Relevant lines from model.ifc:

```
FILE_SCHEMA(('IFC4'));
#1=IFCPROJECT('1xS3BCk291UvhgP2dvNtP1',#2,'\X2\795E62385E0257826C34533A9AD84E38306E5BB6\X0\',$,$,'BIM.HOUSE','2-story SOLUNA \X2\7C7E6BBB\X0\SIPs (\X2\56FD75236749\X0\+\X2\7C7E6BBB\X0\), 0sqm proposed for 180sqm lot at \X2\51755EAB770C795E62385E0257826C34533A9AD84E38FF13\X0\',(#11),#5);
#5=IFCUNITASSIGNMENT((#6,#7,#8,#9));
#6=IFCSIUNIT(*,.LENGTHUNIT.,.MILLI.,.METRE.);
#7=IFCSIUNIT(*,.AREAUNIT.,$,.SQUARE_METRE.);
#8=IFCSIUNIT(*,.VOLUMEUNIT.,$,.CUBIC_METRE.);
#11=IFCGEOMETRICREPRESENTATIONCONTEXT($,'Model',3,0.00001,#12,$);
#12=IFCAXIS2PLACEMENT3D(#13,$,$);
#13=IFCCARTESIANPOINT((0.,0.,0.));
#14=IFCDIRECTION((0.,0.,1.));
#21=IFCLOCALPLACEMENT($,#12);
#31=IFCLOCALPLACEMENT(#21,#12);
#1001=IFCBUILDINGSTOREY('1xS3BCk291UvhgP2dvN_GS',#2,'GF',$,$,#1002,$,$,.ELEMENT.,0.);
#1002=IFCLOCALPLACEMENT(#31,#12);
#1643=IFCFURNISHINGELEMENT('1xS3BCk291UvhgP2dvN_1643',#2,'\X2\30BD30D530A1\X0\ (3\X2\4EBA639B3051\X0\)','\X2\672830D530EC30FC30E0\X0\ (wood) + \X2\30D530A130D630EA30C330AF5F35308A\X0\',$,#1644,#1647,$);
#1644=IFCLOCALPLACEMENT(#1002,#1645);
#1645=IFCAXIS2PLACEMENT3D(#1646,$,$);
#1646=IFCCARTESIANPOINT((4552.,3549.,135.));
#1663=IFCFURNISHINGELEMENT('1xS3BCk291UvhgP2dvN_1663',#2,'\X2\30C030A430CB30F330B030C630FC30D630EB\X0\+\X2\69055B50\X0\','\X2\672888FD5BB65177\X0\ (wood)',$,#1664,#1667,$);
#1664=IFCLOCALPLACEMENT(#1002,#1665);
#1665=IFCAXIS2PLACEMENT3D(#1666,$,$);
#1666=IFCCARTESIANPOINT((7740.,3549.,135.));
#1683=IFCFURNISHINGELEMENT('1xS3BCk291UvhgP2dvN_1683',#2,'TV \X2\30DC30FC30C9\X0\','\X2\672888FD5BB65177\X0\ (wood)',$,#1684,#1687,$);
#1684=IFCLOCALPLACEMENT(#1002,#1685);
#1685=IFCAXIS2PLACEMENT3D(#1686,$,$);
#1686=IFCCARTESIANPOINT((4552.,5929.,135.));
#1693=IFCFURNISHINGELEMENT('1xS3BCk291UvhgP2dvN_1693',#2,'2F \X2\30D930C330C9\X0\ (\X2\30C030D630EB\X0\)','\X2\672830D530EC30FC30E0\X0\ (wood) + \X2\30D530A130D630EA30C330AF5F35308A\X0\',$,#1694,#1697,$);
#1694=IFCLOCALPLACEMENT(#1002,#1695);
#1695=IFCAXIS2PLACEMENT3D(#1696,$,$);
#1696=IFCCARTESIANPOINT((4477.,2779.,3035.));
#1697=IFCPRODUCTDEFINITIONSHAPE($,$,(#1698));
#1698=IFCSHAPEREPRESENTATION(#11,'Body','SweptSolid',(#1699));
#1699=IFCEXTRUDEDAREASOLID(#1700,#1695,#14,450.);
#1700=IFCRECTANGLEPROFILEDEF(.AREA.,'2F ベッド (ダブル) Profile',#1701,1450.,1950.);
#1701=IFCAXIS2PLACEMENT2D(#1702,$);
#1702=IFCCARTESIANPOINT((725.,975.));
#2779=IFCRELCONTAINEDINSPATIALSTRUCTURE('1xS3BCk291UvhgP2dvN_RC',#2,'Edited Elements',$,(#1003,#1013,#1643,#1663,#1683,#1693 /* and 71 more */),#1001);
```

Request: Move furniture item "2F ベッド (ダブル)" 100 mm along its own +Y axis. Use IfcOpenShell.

```python
import ifcopenshell
import ifcopenshell.api.geometry
import ifcopenshell.util.placement
import ifcopenshell.util.unit

model = ifcopenshell.open("model.ifc")
unit_scale = ifcopenshell.util.unit.calculate_unit_scale(model)

item = model.by_guid("1xS3BCk291UvhgP2dvN_1693")
matrix = ifcopenshell.util.placement.get_local_placement(item.ObjectPlacement)
matrix[:3, 3] += matrix[:3, 1] * 0.1 / unit_scale
ifcopenshell.api.geometry.edit_object_placement(model, product=item, matrix=matrix, is_si=False)

print(ifcopenshell.util.placement.get_local_placement(item.ObjectPlacement).round(3) + 0.0)

model.write("model_updated.ifc")
```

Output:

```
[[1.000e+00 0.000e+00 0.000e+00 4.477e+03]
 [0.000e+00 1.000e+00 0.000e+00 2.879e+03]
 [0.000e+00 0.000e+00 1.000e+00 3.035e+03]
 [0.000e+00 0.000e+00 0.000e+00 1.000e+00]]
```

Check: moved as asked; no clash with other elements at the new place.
